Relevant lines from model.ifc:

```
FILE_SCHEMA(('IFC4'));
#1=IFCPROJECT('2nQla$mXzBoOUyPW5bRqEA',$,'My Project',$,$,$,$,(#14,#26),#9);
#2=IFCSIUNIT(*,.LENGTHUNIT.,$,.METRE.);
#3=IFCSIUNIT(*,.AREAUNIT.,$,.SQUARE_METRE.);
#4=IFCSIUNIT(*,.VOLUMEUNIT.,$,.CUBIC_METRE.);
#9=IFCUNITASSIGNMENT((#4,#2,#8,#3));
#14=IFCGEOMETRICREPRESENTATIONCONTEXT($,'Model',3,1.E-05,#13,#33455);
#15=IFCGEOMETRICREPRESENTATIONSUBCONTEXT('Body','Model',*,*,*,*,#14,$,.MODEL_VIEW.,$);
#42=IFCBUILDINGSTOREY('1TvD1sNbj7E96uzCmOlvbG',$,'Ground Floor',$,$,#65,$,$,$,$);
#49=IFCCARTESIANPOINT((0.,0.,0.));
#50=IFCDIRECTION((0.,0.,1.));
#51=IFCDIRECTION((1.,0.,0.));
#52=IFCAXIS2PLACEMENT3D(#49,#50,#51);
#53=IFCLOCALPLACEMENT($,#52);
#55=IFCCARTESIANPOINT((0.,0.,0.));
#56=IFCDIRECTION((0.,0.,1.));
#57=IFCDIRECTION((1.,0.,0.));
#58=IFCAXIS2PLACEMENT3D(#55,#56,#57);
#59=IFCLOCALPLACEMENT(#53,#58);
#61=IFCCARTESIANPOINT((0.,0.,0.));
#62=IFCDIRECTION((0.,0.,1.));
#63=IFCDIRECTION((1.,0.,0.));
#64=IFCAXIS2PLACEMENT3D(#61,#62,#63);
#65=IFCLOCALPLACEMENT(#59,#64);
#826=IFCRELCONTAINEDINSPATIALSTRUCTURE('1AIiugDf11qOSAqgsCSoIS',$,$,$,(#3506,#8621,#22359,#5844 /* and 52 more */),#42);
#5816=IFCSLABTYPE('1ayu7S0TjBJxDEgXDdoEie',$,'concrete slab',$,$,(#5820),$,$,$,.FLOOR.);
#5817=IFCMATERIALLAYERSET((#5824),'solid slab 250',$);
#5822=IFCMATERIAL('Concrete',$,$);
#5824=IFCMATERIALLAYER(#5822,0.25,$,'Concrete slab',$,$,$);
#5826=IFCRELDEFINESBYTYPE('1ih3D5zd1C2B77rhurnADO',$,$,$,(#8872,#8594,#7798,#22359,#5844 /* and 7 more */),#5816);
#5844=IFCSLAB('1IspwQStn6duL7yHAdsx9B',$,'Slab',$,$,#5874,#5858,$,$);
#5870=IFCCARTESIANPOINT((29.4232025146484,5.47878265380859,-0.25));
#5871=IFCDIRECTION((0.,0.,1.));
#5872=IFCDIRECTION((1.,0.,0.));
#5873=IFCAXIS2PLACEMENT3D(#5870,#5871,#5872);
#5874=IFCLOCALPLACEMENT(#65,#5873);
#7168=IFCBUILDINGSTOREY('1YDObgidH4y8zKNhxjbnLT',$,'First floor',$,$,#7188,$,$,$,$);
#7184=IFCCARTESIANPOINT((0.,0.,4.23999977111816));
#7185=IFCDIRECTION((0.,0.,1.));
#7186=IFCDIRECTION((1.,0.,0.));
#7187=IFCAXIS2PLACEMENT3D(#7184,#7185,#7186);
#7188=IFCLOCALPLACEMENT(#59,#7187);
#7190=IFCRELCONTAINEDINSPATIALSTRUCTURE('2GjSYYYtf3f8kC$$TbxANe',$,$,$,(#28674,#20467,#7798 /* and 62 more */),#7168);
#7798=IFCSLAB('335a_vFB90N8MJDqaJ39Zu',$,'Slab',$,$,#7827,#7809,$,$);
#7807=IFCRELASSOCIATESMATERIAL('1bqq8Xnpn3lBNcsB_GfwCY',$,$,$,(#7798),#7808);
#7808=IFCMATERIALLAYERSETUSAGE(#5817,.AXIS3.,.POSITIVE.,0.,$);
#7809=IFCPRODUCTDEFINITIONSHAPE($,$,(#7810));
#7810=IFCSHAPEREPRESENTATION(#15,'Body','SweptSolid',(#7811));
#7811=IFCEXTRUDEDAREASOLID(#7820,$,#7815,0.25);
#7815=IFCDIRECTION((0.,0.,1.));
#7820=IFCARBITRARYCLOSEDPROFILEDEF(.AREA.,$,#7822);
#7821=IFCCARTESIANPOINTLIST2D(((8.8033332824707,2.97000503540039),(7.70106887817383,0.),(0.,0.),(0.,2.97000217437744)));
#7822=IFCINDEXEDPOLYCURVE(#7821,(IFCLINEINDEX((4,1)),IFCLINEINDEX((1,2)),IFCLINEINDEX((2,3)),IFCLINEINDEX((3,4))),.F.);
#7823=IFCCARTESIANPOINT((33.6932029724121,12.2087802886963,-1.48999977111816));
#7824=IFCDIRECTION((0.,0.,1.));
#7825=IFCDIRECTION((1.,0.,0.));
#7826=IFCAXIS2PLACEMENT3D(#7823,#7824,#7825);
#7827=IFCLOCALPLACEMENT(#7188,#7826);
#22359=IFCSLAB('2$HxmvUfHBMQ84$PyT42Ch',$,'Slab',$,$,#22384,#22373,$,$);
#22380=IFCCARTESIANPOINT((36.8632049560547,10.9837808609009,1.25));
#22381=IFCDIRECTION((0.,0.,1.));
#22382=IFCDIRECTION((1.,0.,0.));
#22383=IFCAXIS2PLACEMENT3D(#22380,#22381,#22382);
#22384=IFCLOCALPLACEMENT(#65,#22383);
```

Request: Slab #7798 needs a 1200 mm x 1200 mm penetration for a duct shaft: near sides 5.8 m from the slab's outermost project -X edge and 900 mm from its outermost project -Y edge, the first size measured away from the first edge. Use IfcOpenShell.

```python
import numpy as np
import ifcopenshell
import ifcopenshell.api.feature
import ifcopenshell.api.geometry
import ifcopenshell.api.root
import ifcopenshell.geom
import ifcopenshell.util.placement
import ifcopenshell.util.representation
import ifcopenshell.util.shape
import ifcopenshell.util.unit

model = ifcopenshell.open("model.ifc")
unit_scale = ifcopenshell.util.unit.calculate_unit_scale(model)
settings = ifcopenshell.geom.settings()


def volume(element):
    """Net volume in cubic metres, openings subtracted."""
    shape = ifcopenshell.geom.create_shape(settings, element)
    return ifcopenshell.util.shape.get_volume(shape.geometry)


slab = model.by_guid("335a_vFB90N8MJDqaJ39Zu")
before = volume(slab)

# Extent in the slab's own axes, in metres. The edges named are its -X and -Y sides.
slab_shape = ifcopenshell.geom.create_shape(settings, slab)
vertices = ifcopenshell.util.shape.get_vertices(slab_shape.geometry)
x_min, y_min, bottom = vertices.min(axis=0)
top = vertices[:, 2].max()

opening = ifcopenshell.api.root.create_entity(model, ifc_class="IfcOpeningElement", name="Duct shaft opening", predefined_type="OPENING")
context = ifcopenshell.util.representation.get_context(model, "Model", "Body", "MODEL_VIEW")
width, depth = 1.2, 1.2
outline = [(0.0, 0.0), (width, 0.0), (width, depth), (0.0, depth), (0.0, 0.0)]
# Overshoot both faces by 50 mm so the cut is clean.
shape = ifcopenshell.api.geometry.add_slab_representation(
    model, context=context, depth=top - bottom + 0.1, polyline=outline
)
ifcopenshell.api.geometry.assign_representation(model, product=opening, representation=shape)

matrix = ifcopenshell.util.placement.get_local_placement(slab.ObjectPlacement)
matrix[:, 3] = matrix @ np.append(np.array([x_min + 5.8, y_min + 0.9, bottom - 0.05]) / unit_scale, 1.0)
ifcopenshell.api.geometry.edit_object_placement(model, product=opening, matrix=matrix, is_si=False)
ifcopenshell.api.feature.add_feature(model, feature=opening, element=slab)

after = volume(slab)

print(f"slab volume {before:.3f} -> {after:.3f} m3")

model.write("model_rev.ifc")
```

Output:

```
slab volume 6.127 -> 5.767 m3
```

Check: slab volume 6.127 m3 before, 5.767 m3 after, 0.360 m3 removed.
